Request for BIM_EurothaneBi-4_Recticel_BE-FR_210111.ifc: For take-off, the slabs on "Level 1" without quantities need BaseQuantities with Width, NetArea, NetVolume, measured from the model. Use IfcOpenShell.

First a look at what the model holds.

```python
import ifcopenshell
import ifcopenshell.util.element
import ifcopenshell.util.unit

model = ifcopenshell.open("BIM_EurothaneBi-4_Recticel_BE-FR_210111.ifc")
print(model.schema)
for unit_type in ("LENGTHUNIT", "AREAUNIT", "VOLUMEUNIT"):
    print(unit_type, ifcopenshell.util.unit.calculate_unit_scale(model, unit_type))
storey = next(s for s in model.by_type("IfcBuildingStorey") if s.Name == "Level 1")
slabs = [e for e in ifcopenshell.util.element.get_decomposition(storey) if e.is_a("IfcSlab")]
for e in sorted(slabs, key=lambda e: e.id()):
    print(e.id(), e.is_a(), e.Name, list(ifcopenshell.util.element.get_psets(e, qtos_only=True)), sep=" | ")
```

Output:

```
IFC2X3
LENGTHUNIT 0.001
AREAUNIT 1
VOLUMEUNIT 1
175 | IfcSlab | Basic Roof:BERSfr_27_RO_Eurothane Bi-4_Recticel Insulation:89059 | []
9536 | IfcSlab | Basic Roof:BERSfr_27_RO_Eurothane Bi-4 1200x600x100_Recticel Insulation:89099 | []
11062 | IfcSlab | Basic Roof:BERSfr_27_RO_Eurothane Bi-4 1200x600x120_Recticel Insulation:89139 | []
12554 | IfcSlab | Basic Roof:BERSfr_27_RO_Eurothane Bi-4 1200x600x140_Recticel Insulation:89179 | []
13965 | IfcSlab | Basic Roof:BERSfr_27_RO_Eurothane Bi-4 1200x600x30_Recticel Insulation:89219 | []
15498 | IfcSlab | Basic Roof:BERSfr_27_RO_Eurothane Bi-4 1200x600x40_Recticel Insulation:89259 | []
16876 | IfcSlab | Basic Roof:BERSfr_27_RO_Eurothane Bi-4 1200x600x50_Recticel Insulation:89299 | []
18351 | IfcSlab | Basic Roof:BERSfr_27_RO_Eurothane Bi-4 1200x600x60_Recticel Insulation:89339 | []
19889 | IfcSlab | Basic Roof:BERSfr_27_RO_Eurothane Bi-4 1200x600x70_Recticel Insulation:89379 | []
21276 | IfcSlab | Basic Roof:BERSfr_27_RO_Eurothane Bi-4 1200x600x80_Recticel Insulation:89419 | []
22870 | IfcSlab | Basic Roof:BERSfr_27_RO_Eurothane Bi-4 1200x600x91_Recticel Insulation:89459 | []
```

```python
import ifcopenshell
import ifcopenshell.api.pset
import ifcopenshell.geom
import ifcopenshell.util.element
import ifcopenshell.util.shape
import ifcopenshell.util.unit

model = ifcopenshell.open("BIM_EurothaneBi-4_Recticel_BE-FR_210111.ifc")
unit_scale = ifcopenshell.util.unit.calculate_unit_scale(model)
area_scale = ifcopenshell.util.unit.calculate_unit_scale(model, "AREAUNIT")
volume_scale = ifcopenshell.util.unit.calculate_unit_scale(model, "VOLUMEUNIT")
settings = ifcopenshell.geom.settings()

storey = next(s for s in model.by_type("IfcBuildingStorey") if s.Name == "Level 1")
slabs = [e for e in ifcopenshell.util.element.get_decomposition(storey) if e.is_a("IfcSlab")]

for e in sorted(slabs, key=lambda e: e.id()):
    if ifcopenshell.util.element.get_psets(e, qtos_only=True, should_inherit=False):
        continue
    # Geometry comes back in metres, in the element's own axes.
    shape = ifcopenshell.geom.create_shape(settings, e)
    values = {
        "Width": ifcopenshell.util.shape.get_z(shape.geometry) / unit_scale,
        "NetArea": ifcopenshell.util.shape.get_footprint_area(shape.geometry) / area_scale,
        "NetVolume": ifcopenshell.util.shape.get_volume(shape.geometry) / volume_scale,
    }
    qto = ifcopenshell.api.pset.add_qto(model, product=e, name="BaseQuantities")
    ifcopenshell.api.pset.edit_qto(model, qto=qto, properties=values)
    print(e.id(), {k: round(v, 3) for k, v in values.items()})

model.write("BIM_EurothaneBi-4_Recticel_BE-FR_210111_v2.ifc")
```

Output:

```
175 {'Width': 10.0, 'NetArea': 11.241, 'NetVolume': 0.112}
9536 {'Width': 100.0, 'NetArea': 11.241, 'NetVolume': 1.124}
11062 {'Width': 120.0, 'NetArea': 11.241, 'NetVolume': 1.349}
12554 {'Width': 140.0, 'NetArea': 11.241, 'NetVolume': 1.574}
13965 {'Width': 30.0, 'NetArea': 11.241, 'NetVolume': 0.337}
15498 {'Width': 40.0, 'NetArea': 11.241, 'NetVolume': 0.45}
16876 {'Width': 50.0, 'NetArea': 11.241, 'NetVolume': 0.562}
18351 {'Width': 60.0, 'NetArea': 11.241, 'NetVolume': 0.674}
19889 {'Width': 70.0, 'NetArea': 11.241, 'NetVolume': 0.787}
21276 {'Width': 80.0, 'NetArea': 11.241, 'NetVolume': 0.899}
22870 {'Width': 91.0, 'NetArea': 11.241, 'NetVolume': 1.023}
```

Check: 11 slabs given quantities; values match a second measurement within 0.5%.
